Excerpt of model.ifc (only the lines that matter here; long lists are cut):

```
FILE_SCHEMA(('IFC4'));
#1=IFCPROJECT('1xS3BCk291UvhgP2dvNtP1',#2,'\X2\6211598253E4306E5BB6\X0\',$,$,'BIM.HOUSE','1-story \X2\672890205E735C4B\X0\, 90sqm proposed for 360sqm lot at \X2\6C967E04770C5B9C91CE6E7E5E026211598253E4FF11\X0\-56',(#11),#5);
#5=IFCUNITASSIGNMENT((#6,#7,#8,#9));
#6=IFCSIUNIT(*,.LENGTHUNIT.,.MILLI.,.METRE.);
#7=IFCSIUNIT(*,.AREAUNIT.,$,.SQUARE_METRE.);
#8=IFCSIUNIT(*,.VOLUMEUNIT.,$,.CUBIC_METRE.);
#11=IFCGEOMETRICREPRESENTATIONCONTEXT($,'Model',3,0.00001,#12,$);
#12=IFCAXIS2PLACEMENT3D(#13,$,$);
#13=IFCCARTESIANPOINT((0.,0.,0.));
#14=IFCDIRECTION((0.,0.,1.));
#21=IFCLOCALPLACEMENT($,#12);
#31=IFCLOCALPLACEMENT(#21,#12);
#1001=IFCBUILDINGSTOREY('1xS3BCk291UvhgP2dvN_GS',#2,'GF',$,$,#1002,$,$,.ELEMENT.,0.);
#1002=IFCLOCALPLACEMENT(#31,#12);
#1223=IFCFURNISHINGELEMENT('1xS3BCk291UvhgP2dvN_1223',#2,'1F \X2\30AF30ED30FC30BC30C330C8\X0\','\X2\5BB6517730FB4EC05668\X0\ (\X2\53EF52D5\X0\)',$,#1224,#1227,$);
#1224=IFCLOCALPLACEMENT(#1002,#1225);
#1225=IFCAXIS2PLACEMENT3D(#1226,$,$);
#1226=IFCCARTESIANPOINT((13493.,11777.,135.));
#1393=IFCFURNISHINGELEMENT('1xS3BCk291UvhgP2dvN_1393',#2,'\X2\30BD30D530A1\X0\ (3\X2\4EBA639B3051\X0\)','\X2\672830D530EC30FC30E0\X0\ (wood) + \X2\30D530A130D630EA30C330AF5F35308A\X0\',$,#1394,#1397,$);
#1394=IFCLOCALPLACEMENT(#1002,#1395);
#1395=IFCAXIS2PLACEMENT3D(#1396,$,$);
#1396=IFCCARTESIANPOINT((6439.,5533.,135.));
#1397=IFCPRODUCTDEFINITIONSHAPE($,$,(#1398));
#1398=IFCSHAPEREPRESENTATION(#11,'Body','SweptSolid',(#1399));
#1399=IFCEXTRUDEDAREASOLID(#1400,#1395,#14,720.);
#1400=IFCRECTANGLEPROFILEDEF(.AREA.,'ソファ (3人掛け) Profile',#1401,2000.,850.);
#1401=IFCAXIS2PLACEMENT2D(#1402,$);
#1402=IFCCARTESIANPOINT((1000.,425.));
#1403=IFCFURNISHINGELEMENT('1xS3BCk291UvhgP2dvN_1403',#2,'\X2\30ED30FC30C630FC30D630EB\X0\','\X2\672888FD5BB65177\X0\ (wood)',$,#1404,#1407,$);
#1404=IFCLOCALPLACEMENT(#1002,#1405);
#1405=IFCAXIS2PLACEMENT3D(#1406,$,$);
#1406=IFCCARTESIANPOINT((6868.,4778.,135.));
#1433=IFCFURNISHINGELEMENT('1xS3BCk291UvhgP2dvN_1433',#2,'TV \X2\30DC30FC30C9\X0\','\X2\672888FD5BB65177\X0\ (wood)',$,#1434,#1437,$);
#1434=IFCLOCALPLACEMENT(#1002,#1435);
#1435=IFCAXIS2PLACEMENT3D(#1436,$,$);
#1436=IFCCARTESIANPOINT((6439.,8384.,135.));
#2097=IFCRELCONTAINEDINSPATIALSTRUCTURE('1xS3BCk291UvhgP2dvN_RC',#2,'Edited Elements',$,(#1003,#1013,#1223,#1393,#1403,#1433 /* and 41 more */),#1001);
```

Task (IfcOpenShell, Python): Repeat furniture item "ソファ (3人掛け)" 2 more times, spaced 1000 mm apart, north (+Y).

```python
import numpy as np
import ifcopenshell
import ifcopenshell.api.geometry
import ifcopenshell.api.root
import ifcopenshell.util.element
import ifcopenshell.util.placement

model = ifcopenshell.open("model.ifc")


def reuse_history(source, copy):
    """copy_class also copies each property set's owner history, people and application; keep the originals."""
    for rel in copy.IsDefinedBy:
        if rel.is_a("IfcRelDefinesByProperties") and (history := rel.RelatingPropertyDefinition.OwnerHistory):
            rel.RelatingPropertyDefinition.OwnerHistory = source.OwnerHistory
            ifcopenshell.util.element.remove_deep2(model, history)


source = model.by_guid("1xS3BCk291UvhgP2dvN_1393")
base = ifcopenshell.util.placement.get_local_placement(source.ObjectPlacement)
step = np.array([0.0, 1.0, 0.0]) * 1000.0

for i in range(1, 3):
    copy = ifcopenshell.api.root.copy_class(model, product=source)
    copy.Representation = ifcopenshell.util.element.copy_deep(
        model, source.Representation, exclude=["IfcGeometricRepresentationContext", "IfcRepresentationMap"]
    )
    reuse_history(source, copy)
    matrix = base.copy()
    matrix[:3, 3] += i * step
    print("added at", matrix[:3, 3].round(3) + 0.0)
    ifcopenshell.api.geometry.edit_object_placement(model, product=copy, matrix=matrix, is_si=False)

model.write("model_edited.ifc")
```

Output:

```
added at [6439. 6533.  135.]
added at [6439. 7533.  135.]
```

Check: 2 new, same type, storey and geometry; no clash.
